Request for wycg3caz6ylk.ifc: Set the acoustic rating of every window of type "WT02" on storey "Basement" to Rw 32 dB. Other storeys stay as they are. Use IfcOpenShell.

First a look at what the model holds.

```python
import ifcopenshell
import ifcopenshell.util.element

model = ifcopenshell.open("wycg3caz6ylk.ifc")
print(model.schema)
storey = next(s for s in model.by_type("IfcBuildingStorey") if s.Name == "Basement")
windows = [e for e in ifcopenshell.util.element.get_decomposition(storey) if e.is_a("IfcWindow")]
seen = {}
for e in windows:
    element_type = ifcopenshell.util.element.get_type(e)
    key = (element_type.Name if element_type != e and element_type else None, ifcopenshell.util.element.get_pset(e, "Pset_WindowCommon", "AcousticRating"))
    seen[key] = seen.get(key, 0) + 1
for (name, value), count in sorted(seen.items(), key=str):
    print(count, "x", name, "|", value)
```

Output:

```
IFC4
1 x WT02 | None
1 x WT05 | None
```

```python
import ifcopenshell
import ifcopenshell.api.pset
import ifcopenshell.util.element

model = ifcopenshell.open("wycg3caz6ylk.ifc")

storey = next(s for s in model.by_type("IfcBuildingStorey") if s.Name == "Basement")
windows = [e for e in ifcopenshell.util.element.get_decomposition(storey) if e.is_a("IfcWindow")]

count = 0
for e in windows:
    element_type = ifcopenshell.util.element.get_type(e)
    if element_type in (None, e) or element_type.Name != "WT02":
        continue
    # add_pset returns the element's existing set when there is one.
    pset = ifcopenshell.api.pset.add_pset(model, product=e, name="Pset_WindowCommon")
    ifcopenshell.api.pset.edit_pset(model, pset=pset, properties={"AcousticRating": "Rw 32 dB"})
    count += 1

print(count, "windows updated")

model.write("wycg3caz6ylk-out.ifc")
```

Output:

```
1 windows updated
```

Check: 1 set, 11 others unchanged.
